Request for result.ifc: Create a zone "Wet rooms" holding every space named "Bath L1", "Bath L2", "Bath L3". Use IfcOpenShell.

First a look at what the model holds.

```python
import ifcopenshell

model = ifcopenshell.open("result.ifc")
print(model.schema)
seen = {}
for space in model.by_type("IfcSpace"):
    seen[space.Name] = seen.get(space.Name, 0) + 1
for name, count in sorted(seen.items(), key=str):
    print(count, "x", name)
print("zones:", [z.Name for z in model.by_type("IfcZone")][:20])
```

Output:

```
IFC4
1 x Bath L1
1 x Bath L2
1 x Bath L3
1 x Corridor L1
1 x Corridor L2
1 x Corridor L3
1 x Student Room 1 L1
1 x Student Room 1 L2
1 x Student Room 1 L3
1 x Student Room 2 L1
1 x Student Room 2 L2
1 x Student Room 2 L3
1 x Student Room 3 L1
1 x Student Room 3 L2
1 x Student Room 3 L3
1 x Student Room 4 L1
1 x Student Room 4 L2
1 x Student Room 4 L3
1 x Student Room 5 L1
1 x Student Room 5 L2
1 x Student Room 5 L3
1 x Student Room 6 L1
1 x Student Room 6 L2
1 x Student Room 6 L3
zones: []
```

```python
import ifcopenshell
import ifcopenshell.api.group
import ifcopenshell.api.root

model = ifcopenshell.open("result.ifc")

names = {"Bath L1", "Bath L2", "Bath L3"}
spaces = [s for s in model.by_type("IfcSpace") if s.Name in names]

zone = ifcopenshell.api.root.create_entity(model, ifc_class="IfcZone", name="Wet rooms")
ifcopenshell.api.group.assign_group(model, products=spaces, group=zone)
print(len(spaces), "spaces in", zone.Name)

model.write("result-out.ifc")
```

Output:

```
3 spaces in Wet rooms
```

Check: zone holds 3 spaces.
